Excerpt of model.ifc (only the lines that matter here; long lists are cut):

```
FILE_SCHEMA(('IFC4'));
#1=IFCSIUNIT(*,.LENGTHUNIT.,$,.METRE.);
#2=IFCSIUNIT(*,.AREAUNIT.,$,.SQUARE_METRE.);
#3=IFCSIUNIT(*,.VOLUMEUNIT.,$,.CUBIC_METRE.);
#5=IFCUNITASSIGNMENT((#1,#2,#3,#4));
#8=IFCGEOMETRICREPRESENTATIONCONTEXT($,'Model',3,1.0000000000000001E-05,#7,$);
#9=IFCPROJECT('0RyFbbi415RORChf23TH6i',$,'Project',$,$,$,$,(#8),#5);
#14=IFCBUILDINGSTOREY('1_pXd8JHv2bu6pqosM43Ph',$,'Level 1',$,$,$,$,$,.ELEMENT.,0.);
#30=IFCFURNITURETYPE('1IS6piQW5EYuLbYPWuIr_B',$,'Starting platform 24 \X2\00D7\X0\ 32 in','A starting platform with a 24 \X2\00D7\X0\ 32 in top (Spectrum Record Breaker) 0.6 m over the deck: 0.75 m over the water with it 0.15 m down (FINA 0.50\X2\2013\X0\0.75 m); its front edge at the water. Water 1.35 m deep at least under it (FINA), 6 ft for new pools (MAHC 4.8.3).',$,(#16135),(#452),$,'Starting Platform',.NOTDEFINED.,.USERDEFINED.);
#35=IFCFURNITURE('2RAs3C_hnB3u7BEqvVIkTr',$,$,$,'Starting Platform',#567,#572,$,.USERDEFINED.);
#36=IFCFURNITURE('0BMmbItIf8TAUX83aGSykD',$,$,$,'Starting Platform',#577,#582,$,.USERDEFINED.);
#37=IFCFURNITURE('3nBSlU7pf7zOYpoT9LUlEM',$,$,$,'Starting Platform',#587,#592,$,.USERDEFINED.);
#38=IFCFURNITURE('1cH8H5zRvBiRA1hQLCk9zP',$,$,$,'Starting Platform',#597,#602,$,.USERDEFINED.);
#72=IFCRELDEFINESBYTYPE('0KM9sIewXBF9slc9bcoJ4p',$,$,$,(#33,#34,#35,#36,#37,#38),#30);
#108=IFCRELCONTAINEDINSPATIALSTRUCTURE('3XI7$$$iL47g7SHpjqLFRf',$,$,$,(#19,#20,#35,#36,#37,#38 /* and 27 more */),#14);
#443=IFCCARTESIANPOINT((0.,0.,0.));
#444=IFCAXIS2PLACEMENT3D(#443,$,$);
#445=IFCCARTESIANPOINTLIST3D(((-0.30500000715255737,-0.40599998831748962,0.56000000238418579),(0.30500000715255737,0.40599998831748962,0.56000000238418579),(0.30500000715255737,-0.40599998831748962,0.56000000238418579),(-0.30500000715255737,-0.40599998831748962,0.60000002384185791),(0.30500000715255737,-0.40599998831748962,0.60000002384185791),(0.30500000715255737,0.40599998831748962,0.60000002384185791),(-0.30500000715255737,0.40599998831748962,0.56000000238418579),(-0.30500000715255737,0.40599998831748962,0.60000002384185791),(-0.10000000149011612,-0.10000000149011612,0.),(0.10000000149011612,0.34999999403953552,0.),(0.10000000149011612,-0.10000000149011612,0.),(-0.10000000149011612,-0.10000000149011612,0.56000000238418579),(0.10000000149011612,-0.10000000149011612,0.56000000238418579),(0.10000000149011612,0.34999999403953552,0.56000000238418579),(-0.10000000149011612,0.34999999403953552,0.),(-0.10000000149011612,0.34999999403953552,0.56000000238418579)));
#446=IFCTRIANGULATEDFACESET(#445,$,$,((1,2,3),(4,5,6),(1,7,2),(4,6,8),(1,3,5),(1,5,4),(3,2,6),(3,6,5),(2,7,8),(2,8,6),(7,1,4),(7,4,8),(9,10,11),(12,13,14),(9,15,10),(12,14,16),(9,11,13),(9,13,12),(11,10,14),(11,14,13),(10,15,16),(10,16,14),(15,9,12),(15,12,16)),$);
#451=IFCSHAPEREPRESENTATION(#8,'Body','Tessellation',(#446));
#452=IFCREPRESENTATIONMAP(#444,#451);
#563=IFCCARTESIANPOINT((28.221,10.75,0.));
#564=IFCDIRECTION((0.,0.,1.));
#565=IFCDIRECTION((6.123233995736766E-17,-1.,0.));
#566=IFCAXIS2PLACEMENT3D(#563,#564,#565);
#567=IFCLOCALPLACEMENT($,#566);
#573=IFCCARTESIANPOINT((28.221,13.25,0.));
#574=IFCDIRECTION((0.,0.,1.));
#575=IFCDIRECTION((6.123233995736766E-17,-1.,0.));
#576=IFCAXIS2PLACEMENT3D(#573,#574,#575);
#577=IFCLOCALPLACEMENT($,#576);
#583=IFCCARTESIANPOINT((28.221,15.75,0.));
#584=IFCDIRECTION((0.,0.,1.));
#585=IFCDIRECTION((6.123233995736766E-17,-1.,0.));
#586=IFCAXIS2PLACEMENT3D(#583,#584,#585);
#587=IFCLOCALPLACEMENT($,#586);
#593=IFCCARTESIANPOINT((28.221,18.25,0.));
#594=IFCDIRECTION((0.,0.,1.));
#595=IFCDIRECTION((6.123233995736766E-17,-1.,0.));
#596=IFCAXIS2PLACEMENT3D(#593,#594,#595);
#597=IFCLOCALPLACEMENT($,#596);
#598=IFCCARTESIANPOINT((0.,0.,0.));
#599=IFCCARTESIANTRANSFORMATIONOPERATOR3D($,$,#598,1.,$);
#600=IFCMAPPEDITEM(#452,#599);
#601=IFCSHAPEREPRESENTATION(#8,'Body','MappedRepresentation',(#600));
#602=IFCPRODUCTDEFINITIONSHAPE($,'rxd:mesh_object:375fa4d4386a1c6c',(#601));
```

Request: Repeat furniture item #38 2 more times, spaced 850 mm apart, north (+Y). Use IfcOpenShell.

```python
import numpy as np
import ifcopenshell
import ifcopenshell.api.geometry
import ifcopenshell.api.root
import ifcopenshell.util.element
import ifcopenshell.util.placement

model = ifcopenshell.open("model.ifc")

source = model.by_guid("1cH8H5zRvBiRA1hQLCk9zP")
base = ifcopenshell.util.placement.get_local_placement(source.ObjectPlacement)
step = np.array([0.0, 1.0, 0.0]) * 0.85

for i in range(1, 3):
    copy = ifcopenshell.api.root.copy_class(model, product=source)
    copy.Representation = ifcopenshell.util.element.copy_deep(
        model, source.Representation, exclude=["IfcGeometricRepresentationContext", "IfcRepresentationMap"]
    )
    matrix = base.copy()
    matrix[:3, 3] += i * step
    print("added at", matrix[:3, 3].round(3) + 0.0)
    ifcopenshell.api.geometry.edit_object_placement(model, product=copy, matrix=matrix, is_si=False)

model.write("model-out.ifc")
```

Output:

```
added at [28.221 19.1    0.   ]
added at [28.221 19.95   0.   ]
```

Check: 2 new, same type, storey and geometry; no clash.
